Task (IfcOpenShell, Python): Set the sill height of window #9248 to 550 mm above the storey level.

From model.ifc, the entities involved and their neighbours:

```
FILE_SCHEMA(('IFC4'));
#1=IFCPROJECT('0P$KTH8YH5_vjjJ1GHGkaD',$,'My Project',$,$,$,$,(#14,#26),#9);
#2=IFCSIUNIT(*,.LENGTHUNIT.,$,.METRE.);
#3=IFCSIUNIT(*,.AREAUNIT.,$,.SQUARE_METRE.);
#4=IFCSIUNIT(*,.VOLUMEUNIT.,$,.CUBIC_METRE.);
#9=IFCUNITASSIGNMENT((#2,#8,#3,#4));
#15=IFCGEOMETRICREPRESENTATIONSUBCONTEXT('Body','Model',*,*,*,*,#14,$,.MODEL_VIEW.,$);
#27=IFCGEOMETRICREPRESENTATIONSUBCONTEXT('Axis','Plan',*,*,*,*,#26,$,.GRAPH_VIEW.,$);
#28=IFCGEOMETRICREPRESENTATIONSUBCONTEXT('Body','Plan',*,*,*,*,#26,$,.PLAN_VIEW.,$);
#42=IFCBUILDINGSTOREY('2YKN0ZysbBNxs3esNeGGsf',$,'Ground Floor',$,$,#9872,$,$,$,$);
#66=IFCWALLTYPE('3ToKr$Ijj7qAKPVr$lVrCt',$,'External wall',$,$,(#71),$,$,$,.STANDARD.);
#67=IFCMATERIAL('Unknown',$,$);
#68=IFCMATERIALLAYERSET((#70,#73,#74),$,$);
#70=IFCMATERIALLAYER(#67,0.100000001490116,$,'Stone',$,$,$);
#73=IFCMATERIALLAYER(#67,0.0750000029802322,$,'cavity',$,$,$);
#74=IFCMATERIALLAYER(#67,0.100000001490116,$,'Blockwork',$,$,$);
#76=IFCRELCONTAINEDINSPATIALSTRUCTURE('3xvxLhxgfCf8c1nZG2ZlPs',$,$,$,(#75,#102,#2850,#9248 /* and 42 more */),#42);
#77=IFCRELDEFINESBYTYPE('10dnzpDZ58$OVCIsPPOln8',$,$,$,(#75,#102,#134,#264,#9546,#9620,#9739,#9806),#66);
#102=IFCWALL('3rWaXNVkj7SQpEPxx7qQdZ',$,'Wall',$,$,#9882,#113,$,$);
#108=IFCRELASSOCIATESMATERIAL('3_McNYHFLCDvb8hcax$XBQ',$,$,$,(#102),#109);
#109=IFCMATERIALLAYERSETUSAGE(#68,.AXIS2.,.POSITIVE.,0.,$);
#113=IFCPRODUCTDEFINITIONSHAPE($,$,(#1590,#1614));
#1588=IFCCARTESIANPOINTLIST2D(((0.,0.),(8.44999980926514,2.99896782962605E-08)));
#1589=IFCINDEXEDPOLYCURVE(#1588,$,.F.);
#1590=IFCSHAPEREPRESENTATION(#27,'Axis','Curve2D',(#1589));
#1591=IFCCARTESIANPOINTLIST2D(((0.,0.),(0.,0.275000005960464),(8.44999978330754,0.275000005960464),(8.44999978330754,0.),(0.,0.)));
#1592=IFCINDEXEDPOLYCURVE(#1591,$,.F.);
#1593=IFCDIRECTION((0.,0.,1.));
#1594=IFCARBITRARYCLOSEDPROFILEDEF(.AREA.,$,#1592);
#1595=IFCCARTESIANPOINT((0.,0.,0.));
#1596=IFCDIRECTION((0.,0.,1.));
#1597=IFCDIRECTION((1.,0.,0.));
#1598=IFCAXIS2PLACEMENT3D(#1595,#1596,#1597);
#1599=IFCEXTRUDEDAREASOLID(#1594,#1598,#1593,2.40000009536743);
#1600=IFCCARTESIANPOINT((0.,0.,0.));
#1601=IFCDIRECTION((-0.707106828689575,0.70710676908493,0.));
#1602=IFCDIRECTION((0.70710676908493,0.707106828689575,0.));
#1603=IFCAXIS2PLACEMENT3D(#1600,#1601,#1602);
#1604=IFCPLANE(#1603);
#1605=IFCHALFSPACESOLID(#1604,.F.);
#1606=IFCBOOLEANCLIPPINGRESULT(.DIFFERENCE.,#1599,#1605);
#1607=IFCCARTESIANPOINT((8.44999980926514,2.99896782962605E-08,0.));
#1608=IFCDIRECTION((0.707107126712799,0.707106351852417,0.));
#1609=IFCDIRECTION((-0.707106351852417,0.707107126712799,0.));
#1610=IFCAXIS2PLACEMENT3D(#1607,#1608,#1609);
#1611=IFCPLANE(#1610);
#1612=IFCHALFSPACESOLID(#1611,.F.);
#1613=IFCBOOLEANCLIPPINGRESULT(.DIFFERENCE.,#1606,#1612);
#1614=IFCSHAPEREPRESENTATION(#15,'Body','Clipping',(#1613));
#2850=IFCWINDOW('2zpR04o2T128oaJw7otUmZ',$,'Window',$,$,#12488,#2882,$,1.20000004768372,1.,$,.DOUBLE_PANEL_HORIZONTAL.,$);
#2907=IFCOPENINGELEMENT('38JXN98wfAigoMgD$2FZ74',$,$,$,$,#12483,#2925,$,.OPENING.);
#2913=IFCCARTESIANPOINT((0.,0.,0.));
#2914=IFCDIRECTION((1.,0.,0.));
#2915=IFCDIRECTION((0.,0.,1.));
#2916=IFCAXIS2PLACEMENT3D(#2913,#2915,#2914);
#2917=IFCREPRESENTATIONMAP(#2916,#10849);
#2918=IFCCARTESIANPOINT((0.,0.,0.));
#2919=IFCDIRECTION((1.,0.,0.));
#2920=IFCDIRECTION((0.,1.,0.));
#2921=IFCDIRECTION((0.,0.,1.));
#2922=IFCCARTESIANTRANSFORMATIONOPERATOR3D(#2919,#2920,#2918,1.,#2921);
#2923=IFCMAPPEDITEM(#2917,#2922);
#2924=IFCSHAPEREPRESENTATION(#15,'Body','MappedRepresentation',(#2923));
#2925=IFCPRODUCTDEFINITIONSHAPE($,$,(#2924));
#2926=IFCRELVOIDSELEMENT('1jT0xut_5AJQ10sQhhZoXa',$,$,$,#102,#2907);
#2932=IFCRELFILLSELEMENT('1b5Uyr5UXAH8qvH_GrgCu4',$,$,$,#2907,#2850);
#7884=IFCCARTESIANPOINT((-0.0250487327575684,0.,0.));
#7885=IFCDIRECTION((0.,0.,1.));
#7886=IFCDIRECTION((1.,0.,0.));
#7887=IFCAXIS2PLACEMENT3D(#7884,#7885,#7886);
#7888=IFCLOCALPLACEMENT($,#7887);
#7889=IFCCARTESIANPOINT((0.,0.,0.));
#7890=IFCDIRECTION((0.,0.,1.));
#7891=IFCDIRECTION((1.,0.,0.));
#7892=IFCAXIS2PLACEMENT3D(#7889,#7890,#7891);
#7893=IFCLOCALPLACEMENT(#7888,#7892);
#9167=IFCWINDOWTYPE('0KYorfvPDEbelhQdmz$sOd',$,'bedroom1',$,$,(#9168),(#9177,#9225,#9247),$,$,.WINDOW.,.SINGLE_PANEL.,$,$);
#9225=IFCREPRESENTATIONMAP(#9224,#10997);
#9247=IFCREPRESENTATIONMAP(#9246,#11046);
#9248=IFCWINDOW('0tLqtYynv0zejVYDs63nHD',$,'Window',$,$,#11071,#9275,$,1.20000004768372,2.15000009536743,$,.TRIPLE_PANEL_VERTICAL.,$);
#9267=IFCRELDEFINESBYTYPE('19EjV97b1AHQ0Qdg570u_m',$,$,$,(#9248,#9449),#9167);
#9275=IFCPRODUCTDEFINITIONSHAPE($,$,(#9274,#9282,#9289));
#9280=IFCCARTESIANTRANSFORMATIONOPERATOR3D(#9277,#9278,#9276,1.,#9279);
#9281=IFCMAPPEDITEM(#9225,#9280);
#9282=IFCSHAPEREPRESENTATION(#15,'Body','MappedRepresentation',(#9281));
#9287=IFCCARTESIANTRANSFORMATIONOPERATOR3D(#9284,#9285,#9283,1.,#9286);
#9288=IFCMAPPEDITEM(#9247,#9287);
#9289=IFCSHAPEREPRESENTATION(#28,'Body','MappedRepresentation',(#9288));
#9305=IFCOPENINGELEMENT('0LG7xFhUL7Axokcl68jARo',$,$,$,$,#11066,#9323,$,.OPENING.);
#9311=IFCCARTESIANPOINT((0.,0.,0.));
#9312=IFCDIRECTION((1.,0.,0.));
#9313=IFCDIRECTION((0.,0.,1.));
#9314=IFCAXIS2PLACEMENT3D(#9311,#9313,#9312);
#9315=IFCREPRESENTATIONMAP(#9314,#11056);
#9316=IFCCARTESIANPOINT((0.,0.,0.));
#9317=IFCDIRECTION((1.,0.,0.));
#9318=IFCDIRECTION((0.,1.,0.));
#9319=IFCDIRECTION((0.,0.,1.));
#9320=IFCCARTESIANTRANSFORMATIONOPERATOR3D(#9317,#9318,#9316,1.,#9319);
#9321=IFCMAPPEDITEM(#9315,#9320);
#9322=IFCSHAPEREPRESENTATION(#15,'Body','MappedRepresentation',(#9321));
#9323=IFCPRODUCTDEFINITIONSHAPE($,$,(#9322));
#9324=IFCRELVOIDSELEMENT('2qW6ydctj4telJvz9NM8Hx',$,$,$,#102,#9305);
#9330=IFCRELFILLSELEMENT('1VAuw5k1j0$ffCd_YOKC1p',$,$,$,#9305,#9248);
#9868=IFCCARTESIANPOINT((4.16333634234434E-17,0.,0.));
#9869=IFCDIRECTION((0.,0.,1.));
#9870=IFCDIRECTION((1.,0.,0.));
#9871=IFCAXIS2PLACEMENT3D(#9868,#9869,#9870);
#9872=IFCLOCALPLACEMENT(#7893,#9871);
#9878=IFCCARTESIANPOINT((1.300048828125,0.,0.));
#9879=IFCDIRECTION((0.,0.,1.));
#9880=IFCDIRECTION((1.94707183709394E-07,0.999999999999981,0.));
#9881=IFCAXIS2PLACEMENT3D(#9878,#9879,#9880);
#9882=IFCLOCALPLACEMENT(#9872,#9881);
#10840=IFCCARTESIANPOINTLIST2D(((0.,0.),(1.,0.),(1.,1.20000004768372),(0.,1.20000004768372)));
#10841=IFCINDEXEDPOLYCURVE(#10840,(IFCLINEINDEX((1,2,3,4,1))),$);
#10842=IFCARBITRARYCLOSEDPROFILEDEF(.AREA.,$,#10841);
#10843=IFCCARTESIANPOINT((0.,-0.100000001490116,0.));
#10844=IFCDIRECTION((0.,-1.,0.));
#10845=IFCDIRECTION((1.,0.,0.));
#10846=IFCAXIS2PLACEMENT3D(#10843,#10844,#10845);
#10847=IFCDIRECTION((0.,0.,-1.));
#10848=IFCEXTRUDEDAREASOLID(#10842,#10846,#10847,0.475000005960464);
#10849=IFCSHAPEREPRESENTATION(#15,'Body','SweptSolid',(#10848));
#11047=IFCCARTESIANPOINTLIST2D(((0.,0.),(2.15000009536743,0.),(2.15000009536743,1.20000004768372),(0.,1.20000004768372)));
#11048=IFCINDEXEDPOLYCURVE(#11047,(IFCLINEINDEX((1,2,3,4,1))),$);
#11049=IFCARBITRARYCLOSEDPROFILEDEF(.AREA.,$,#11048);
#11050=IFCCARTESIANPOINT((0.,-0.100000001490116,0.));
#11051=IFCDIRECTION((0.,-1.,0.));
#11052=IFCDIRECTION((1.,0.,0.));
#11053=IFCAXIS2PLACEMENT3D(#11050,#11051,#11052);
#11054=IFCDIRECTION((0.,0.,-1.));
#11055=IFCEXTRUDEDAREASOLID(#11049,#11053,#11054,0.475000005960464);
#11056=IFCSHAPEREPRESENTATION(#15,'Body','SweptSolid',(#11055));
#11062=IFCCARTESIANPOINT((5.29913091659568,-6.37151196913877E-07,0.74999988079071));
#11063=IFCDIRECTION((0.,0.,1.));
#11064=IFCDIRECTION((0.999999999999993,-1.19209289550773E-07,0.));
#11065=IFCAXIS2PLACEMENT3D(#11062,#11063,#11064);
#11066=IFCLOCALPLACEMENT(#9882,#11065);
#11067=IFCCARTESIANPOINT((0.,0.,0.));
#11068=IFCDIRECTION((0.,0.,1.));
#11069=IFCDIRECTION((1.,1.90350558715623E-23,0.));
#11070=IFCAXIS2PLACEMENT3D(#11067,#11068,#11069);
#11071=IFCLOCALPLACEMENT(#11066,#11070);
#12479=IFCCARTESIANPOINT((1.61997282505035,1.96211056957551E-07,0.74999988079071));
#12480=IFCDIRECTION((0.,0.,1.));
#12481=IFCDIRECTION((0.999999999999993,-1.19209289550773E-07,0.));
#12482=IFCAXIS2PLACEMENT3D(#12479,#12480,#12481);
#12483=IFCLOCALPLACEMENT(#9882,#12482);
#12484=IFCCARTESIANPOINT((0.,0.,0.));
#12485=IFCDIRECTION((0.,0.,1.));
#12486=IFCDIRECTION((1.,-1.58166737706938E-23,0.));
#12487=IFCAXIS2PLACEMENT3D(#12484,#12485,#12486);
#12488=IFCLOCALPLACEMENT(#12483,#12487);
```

```python
import numpy as np
import ifcopenshell
import ifcopenshell.api.geometry
import ifcopenshell.geom
import ifcopenshell.util.element
import ifcopenshell.util.placement
import ifcopenshell.util.shape
import ifcopenshell.util.unit

model = ifcopenshell.open("model.ifc")
unit_scale = ifcopenshell.util.unit.calculate_unit_scale(model)

window = model.by_id(9248)
opening = window.FillsVoids[0].RelatingOpeningElement
storey = ifcopenshell.util.element.get_container(window, ifc_class="IfcBuildingStorey")
level = ifcopenshell.util.placement.get_local_placement(storey.ObjectPlacement)[2, 3]

# The opening's origin need not be at the sill, so measure its lowest point.
shape = ifcopenshell.geom.create_shape(ifcopenshell.geom.settings(), opening)
bottom = ifcopenshell.util.shape.get_shape_bottom_elevation(shape, shape.geometry) / unit_scale
dz = level + 0.55 - bottom

shift = np.array([0.0, 0.0, dz])
# The window is placed relative to its opening, so it follows when the opening moves.
matrix = ifcopenshell.util.placement.get_local_placement(opening.ObjectPlacement)
matrix[:3, 3] += shift
ifcopenshell.api.geometry.edit_object_placement(
    model, product=opening, matrix=matrix, is_si=False, should_transform_children=True
)

print(f"moved by {dz * unit_scale:+.3f} m")

model.write("model-out.ifc")
```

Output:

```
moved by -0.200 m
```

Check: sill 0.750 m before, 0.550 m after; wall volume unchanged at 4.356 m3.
